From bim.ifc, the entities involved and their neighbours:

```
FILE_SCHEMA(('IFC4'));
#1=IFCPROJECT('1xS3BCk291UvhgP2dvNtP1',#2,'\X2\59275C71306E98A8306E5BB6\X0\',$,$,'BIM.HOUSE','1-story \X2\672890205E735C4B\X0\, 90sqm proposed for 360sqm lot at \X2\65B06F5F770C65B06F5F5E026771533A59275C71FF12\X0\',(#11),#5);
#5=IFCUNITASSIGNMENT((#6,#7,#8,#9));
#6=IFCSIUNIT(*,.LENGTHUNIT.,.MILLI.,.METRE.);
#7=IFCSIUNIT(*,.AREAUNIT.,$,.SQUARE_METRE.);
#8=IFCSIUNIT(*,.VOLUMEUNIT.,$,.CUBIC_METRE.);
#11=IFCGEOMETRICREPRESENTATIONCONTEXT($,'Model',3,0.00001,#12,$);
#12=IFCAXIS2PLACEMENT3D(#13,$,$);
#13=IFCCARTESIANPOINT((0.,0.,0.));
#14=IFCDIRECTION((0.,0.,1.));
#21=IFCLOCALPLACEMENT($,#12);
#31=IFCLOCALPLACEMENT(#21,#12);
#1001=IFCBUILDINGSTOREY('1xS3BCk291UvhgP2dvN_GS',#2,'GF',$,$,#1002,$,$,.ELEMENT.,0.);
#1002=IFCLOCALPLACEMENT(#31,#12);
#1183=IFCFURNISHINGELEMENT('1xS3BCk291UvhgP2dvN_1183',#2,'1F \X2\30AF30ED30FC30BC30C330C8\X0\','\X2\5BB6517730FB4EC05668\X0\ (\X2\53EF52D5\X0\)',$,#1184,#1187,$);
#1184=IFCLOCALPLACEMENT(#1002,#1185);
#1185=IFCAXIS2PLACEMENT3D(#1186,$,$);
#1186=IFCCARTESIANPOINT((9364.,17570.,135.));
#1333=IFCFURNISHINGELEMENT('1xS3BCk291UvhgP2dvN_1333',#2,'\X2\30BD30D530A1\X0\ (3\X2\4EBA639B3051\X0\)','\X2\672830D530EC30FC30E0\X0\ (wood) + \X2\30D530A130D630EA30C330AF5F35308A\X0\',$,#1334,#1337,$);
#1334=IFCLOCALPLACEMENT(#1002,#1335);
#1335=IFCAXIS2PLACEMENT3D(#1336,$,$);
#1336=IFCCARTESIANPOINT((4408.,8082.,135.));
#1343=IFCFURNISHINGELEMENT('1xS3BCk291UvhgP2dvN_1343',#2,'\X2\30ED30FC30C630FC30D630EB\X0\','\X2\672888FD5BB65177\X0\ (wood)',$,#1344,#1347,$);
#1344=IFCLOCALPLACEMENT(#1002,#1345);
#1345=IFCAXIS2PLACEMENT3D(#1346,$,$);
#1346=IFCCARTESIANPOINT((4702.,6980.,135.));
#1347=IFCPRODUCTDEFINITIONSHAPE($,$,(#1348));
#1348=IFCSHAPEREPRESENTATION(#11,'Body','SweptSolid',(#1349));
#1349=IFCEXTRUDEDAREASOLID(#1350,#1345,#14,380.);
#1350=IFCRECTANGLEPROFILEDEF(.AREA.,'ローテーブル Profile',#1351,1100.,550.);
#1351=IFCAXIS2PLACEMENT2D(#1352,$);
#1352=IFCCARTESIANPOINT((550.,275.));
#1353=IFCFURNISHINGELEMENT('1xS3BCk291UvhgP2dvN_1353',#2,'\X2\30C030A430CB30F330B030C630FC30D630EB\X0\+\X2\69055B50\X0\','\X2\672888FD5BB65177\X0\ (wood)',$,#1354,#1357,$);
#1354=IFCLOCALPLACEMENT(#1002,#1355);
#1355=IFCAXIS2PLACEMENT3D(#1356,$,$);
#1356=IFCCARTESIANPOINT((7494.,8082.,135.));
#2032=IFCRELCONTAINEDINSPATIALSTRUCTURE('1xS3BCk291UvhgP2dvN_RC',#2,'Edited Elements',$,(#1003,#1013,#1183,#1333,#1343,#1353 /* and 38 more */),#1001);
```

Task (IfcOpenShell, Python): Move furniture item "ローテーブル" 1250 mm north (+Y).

```python
import ifcopenshell
import ifcopenshell.api.geometry
import ifcopenshell.util.placement
import ifcopenshell.util.unit

model = ifcopenshell.open("bim.ifc")
unit_scale = ifcopenshell.util.unit.calculate_unit_scale(model)

item = model.by_guid("1xS3BCk291UvhgP2dvN_1343")
matrix = ifcopenshell.util.placement.get_local_placement(item.ObjectPlacement)
matrix[1, 3] += 1.25 / unit_scale
ifcopenshell.api.geometry.edit_object_placement(model, product=item, matrix=matrix, is_si=False)

print(ifcopenshell.util.placement.get_local_placement(item.ObjectPlacement).round(3) + 0.0)

model.write("bim_edited.ifc")
```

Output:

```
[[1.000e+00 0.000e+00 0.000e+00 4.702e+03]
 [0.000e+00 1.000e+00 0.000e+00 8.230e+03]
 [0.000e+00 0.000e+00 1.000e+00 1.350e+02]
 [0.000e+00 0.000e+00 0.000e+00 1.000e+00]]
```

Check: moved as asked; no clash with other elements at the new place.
